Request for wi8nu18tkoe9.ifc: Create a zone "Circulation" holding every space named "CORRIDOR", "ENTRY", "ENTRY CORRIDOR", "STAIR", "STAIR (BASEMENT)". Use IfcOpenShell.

First a look at what the model holds.

```python
import ifcopenshell

model = ifcopenshell.open("wi8nu18tkoe9.ifc")
print(model.schema)
seen = {}
for space in model.by_type("IfcSpace"):
    seen[space.LongName] = seen.get(space.LongName, 0) + 1
for name, count in sorted(seen.items(), key=str):
    print(count, "x", name)
print("zones:", [z.Name for z in model.by_type("IfcZone")][:20])
```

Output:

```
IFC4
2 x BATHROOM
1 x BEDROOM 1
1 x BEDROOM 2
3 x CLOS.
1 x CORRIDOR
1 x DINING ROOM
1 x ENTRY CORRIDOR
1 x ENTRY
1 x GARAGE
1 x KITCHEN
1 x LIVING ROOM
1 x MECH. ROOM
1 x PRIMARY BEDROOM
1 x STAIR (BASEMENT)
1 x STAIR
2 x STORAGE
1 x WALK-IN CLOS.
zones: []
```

```python
import ifcopenshell
import ifcopenshell.api.group
import ifcopenshell.api.root

model = ifcopenshell.open("wi8nu18tkoe9.ifc")

names = {"CORRIDOR", "ENTRY", "ENTRY CORRIDOR", "STAIR", "STAIR (BASEMENT)"}
spaces = [s for s in model.by_type("IfcSpace") if s.LongName in names]

zone = ifcopenshell.api.root.create_entity(model, ifc_class="IfcZone", name="Circulation")
ifcopenshell.api.group.assign_group(model, products=spaces, group=zone)
print(len(spaces), "spaces in", zone.Name)

model.write("wi8nu18tkoe9_edited.ifc")
```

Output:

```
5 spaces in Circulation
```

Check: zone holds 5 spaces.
